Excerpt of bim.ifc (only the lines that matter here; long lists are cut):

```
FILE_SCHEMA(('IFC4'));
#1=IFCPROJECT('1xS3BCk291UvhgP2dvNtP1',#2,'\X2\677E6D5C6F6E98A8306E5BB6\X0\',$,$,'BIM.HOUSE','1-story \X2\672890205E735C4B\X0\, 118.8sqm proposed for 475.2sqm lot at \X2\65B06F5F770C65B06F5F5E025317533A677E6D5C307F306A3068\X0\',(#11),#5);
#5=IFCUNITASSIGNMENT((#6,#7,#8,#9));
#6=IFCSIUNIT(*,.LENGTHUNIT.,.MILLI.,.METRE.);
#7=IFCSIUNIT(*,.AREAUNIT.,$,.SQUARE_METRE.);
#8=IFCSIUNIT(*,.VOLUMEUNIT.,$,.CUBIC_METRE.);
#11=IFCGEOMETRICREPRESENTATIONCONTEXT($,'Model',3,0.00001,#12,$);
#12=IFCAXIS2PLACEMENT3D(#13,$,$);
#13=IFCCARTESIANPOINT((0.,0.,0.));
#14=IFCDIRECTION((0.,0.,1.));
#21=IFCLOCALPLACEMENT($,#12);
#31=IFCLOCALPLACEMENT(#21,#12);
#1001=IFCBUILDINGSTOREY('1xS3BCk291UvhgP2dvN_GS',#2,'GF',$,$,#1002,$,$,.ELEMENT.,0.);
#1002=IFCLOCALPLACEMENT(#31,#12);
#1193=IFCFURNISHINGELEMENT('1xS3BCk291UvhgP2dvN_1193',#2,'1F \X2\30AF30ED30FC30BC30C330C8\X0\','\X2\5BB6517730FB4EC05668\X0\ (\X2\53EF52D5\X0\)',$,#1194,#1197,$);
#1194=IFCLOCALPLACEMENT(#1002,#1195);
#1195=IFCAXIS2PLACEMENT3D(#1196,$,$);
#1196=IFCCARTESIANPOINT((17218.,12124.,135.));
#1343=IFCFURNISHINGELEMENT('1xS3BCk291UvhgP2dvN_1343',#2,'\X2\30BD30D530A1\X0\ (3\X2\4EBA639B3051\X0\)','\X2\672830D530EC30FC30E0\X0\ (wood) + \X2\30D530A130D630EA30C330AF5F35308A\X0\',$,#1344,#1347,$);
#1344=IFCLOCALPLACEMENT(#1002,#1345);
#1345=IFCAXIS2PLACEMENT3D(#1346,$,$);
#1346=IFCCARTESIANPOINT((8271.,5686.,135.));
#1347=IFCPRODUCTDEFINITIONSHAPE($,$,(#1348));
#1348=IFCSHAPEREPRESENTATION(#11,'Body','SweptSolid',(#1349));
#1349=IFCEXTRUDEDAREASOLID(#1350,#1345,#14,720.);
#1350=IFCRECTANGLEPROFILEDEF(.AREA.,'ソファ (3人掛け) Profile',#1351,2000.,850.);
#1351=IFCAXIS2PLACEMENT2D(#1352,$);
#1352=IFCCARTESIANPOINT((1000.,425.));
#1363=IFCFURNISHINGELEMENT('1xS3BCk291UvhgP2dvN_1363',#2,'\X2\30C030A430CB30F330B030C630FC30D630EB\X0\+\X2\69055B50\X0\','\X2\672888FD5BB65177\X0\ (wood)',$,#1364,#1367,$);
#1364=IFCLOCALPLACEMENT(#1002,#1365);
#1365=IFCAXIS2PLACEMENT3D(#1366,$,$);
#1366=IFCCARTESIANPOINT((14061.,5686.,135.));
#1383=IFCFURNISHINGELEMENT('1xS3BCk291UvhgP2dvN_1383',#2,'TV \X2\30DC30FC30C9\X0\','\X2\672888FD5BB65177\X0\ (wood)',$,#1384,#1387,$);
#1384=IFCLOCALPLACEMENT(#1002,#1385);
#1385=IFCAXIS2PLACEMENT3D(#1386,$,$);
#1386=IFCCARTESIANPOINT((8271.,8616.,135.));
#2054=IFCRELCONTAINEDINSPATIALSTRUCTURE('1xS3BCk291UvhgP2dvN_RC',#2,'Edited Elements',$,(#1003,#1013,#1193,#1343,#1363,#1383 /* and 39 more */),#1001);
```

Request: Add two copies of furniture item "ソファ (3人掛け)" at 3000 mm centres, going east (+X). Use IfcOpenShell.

```python
import numpy as np
import ifcopenshell
import ifcopenshell.api.geometry
import ifcopenshell.api.root
import ifcopenshell.util.element
import ifcopenshell.util.placement

model = ifcopenshell.open("bim.ifc")


def reuse_history(source, copy):
    """copy_class also copies each property set's owner history, people and application; keep the originals."""
    for rel in copy.IsDefinedBy:
        if rel.is_a("IfcRelDefinesByProperties") and (history := rel.RelatingPropertyDefinition.OwnerHistory):
            rel.RelatingPropertyDefinition.OwnerHistory = source.OwnerHistory
            ifcopenshell.util.element.remove_deep2(model, history)


source = model.by_guid("1xS3BCk291UvhgP2dvN_1343")
base = ifcopenshell.util.placement.get_local_placement(source.ObjectPlacement)
step = np.array([1.0, 0.0, 0.0]) * 3000.0

for i in range(1, 3):
    copy = ifcopenshell.api.root.copy_class(model, product=source)
    copy.Representation = ifcopenshell.util.element.copy_deep(
        model, source.Representation, exclude=["IfcGeometricRepresentationContext", "IfcRepresentationMap"]
    )
    reuse_history(source, copy)
    matrix = base.copy()
    matrix[:3, 3] += i * step
    print("added at", matrix[:3, 3].round(3) + 0.0)
    ifcopenshell.api.geometry.edit_object_placement(model, product=copy, matrix=matrix, is_si=False)

model.write("bim-out.ifc")
```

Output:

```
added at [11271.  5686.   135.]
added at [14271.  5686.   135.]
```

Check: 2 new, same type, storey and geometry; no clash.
